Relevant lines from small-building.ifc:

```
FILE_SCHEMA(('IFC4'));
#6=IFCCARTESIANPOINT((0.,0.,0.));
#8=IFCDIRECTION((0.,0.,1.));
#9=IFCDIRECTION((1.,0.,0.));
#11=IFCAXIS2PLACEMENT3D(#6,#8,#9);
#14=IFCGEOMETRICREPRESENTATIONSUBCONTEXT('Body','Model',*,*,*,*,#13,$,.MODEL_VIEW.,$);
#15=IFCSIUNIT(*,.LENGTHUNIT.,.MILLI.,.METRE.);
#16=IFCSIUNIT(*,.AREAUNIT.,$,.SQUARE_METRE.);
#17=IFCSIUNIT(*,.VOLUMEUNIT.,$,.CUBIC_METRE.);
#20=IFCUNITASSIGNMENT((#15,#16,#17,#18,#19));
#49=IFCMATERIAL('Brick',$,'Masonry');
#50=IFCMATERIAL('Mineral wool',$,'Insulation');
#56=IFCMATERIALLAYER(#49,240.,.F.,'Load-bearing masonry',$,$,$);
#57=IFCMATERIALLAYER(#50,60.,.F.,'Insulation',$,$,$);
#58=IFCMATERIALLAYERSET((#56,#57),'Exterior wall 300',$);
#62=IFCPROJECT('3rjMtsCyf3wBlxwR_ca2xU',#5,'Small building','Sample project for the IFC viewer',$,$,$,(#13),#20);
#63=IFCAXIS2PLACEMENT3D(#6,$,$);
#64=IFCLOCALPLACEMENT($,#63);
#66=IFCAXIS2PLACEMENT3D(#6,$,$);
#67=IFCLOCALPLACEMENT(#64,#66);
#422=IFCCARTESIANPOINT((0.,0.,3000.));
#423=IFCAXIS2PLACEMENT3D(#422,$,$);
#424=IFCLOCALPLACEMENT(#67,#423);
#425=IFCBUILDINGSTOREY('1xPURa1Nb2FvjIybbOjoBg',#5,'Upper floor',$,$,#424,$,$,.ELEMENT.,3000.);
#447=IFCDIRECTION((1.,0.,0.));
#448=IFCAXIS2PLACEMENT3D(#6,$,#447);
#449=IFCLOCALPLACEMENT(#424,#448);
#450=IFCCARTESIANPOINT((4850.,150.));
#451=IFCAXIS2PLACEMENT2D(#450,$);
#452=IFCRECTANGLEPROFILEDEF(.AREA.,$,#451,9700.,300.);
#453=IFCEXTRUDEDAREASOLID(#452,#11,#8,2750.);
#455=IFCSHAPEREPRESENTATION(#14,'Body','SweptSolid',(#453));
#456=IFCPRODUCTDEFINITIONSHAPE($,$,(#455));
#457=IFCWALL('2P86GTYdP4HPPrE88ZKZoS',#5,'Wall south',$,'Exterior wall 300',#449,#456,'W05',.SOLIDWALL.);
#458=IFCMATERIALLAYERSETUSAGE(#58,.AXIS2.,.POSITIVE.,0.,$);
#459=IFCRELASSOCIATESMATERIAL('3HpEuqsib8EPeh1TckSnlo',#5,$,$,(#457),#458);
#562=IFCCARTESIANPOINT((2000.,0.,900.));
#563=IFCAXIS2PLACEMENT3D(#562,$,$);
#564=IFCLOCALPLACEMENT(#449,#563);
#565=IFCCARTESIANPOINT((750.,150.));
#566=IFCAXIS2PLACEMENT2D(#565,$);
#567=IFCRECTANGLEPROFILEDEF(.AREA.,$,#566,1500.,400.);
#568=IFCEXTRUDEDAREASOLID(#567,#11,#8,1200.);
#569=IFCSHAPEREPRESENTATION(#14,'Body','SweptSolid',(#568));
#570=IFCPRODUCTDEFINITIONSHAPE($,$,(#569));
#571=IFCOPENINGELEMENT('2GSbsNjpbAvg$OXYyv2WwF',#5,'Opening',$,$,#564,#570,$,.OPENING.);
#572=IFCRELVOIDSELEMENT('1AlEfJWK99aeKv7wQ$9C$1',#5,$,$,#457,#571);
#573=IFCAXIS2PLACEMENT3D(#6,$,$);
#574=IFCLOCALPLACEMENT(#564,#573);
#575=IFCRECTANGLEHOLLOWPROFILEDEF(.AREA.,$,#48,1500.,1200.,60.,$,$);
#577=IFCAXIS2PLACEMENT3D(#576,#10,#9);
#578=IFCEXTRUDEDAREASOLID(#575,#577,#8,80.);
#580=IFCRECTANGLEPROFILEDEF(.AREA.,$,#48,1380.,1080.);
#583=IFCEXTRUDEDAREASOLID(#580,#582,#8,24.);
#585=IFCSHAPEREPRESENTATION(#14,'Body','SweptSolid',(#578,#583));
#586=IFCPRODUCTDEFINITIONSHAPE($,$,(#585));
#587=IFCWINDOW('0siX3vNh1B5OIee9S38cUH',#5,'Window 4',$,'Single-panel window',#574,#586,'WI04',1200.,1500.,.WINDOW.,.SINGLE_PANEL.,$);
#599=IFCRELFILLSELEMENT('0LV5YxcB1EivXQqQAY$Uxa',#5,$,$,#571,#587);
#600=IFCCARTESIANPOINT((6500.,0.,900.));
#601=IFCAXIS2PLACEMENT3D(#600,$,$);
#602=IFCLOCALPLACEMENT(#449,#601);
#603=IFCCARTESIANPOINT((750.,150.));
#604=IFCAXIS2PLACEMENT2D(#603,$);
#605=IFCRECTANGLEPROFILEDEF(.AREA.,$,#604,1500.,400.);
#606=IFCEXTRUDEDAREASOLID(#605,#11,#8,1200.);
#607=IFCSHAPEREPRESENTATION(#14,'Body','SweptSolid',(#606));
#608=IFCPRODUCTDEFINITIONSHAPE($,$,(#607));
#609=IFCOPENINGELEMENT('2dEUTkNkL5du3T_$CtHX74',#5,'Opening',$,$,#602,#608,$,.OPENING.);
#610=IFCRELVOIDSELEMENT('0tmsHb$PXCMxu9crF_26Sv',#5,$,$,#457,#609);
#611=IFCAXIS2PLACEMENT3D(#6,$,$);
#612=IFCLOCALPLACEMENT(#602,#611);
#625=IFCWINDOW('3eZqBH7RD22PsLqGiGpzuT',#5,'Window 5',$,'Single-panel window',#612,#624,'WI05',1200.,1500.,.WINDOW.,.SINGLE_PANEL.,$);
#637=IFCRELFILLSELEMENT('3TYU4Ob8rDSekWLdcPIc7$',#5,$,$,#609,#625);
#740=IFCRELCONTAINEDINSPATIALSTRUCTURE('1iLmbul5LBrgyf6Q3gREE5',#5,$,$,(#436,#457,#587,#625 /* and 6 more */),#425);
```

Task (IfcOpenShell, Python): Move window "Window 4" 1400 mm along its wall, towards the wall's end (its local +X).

```python
import ifcopenshell
import ifcopenshell.api.geometry
import ifcopenshell.util.placement
import ifcopenshell.util.unit

model = ifcopenshell.open("small-building.ifc")
unit_scale = ifcopenshell.util.unit.calculate_unit_scale(model)

window = model.by_guid("0siX3vNh1B5OIee9S38cUH")
opening = window.FillsVoids[0].RelatingOpeningElement
wall = opening.VoidsElements[0].RelatingBuildingElement

wall_matrix = ifcopenshell.util.placement.get_local_placement(wall.ObjectPlacement)
shift = wall_matrix[:3, 0] * 1.4 / unit_scale
before = ifcopenshell.util.placement.get_local_placement(window.ObjectPlacement)[:3, 3].copy()

# The window is placed relative to its opening, so it follows when the opening moves.
matrix = ifcopenshell.util.placement.get_local_placement(opening.ObjectPlacement)
matrix[:3, 3] += shift
ifcopenshell.api.geometry.edit_object_placement(
    model, product=opening, matrix=matrix, is_si=False, should_transform_children=True
)

after = ifcopenshell.util.placement.get_local_placement(window.ObjectPlacement)[:3, 3]
print("window moved by", (after - before).round(3) + 0.0)

model.write("small-building_v2.ifc")
```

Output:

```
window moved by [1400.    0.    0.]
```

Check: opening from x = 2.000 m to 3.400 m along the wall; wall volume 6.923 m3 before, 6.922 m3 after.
